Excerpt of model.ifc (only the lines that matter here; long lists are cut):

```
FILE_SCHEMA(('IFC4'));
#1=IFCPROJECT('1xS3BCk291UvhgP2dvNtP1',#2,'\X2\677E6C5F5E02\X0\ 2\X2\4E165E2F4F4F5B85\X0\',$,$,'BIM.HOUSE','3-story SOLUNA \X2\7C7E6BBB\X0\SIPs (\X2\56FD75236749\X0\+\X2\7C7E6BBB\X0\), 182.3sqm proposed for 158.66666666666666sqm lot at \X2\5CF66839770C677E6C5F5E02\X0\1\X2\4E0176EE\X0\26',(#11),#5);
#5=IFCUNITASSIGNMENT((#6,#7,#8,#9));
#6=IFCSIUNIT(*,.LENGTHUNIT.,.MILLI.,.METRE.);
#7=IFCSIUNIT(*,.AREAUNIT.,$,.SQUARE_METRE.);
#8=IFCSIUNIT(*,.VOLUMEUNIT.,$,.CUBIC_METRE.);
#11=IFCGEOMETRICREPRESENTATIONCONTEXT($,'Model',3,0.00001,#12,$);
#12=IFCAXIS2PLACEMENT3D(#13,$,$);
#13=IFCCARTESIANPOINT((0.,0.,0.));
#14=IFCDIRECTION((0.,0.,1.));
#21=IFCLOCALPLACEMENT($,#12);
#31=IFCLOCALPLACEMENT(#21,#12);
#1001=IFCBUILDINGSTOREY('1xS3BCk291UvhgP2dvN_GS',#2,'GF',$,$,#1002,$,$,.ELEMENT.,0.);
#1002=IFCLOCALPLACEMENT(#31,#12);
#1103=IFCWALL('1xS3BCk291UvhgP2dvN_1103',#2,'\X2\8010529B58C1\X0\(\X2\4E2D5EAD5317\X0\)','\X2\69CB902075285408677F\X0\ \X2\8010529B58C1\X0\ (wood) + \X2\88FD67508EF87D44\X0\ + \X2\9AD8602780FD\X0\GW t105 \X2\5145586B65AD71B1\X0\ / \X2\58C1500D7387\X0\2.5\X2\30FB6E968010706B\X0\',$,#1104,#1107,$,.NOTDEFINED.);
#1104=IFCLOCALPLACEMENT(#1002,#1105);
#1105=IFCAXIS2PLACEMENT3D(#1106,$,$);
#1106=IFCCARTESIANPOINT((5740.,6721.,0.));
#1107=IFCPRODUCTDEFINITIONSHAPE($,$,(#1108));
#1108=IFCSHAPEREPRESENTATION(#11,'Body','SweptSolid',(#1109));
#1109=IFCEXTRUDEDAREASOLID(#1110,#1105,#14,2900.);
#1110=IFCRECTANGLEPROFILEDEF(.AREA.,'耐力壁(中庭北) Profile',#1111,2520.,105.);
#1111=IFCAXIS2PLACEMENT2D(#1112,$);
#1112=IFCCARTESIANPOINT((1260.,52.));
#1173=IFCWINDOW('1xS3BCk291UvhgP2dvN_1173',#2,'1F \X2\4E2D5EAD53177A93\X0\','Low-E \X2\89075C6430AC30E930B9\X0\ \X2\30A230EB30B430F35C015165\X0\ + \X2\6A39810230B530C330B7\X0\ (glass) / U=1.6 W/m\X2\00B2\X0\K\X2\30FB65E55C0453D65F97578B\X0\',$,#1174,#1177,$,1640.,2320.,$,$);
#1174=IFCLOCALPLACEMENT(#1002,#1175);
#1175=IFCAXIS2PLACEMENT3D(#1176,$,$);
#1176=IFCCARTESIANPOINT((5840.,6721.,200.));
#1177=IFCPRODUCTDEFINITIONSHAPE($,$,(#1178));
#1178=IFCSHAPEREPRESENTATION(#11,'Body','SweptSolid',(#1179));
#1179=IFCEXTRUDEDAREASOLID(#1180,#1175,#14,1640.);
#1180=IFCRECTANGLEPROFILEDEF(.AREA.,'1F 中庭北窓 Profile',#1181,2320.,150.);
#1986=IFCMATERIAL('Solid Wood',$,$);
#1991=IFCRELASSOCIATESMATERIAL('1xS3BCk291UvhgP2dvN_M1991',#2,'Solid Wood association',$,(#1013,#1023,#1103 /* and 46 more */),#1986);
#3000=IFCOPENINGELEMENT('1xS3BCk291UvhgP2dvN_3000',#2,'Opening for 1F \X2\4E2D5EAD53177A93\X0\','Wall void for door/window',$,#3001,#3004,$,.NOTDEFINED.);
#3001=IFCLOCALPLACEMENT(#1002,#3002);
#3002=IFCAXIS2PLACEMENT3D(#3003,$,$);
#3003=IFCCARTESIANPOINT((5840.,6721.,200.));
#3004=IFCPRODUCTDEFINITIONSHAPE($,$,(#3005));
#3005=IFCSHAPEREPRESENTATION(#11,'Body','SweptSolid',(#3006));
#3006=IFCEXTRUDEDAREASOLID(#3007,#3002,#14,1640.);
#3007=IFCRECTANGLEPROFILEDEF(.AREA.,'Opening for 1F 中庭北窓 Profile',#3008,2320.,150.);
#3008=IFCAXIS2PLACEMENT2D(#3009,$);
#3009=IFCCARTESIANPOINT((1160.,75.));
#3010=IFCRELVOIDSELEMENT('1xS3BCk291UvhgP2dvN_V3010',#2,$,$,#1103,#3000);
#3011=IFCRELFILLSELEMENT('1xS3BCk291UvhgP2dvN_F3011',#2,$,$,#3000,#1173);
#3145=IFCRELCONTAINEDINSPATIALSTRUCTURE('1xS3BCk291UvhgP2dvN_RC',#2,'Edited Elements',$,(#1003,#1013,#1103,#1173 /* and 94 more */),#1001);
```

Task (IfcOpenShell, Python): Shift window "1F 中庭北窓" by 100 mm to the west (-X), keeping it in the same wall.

```python
import ifcopenshell
import ifcopenshell.api.geometry
import ifcopenshell.util.placement
import ifcopenshell.util.unit

model = ifcopenshell.open("model.ifc")
unit_scale = ifcopenshell.util.unit.calculate_unit_scale(model)

window = model.by_guid("1xS3BCk291UvhgP2dvN_1173")
opening = window.FillsVoids[0].RelatingOpeningElement
wall = opening.VoidsElements[0].RelatingBuildingElement

wall_matrix = ifcopenshell.util.placement.get_local_placement(wall.ObjectPlacement)
shift = wall_matrix[:3, 0] * -0.1 / unit_scale
before = ifcopenshell.util.placement.get_local_placement(window.ObjectPlacement)[:3, 3].copy()

# The window is not placed relative to its opening, so move both.
for product in (opening, window):
    matrix = ifcopenshell.util.placement.get_local_placement(product.ObjectPlacement)
    matrix[:3, 3] += shift
    ifcopenshell.api.geometry.edit_object_placement(model, product=product, matrix=matrix, is_si=False)

after = ifcopenshell.util.placement.get_local_placement(window.ObjectPlacement)[:3, 3]
print("window moved by", (after - before).round(3) + 0.0)

model.write("model_edited.ifc")
```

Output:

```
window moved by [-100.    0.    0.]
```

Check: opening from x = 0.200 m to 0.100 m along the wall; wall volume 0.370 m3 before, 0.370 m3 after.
